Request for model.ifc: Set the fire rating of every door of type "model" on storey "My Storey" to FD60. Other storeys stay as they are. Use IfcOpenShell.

First a look at what the model holds.

```python
import ifcopenshell
import ifcopenshell.util.element

model = ifcopenshell.open("model.ifc")
print(model.schema)
storey = next(s for s in model.by_type("IfcBuildingStorey") if s.Name == "My Storey")
doors = [e for e in ifcopenshell.util.element.get_decomposition(storey) if e.is_a("IfcDoor")]
seen = {}
for e in doors:
    element_type = ifcopenshell.util.element.get_type(e)
    key = (element_type.Name if element_type != e and element_type else None, ifcopenshell.util.element.get_pset(e, "Pset_DoorCommon", "FireRating"))
    seen[key] = seen.get(key, 0) + 1
for (name, value), count in sorted(seen.items(), key=str):
    print(count, "x", name, "|", value)
```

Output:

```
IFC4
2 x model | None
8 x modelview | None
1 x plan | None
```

```python
import ifcopenshell
import ifcopenshell.api.pset
import ifcopenshell.util.element

model = ifcopenshell.open("model.ifc")

storey = next(s for s in model.by_type("IfcBuildingStorey") if s.Name == "My Storey")
doors = [e for e in ifcopenshell.util.element.get_decomposition(storey) if e.is_a("IfcDoor")]

count = 0
for e in doors:
    element_type = ifcopenshell.util.element.get_type(e)
    if element_type in (None, e) or element_type.Name != "model":
        continue
    # add_pset returns the element's existing set when there is one.
    pset = ifcopenshell.api.pset.add_pset(model, product=e, name="Pset_DoorCommon")
    ifcopenshell.api.pset.edit_pset(model, pset=pset, properties={"FireRating": "FD60"})
    count += 1

print(count, "doors updated")

model.write("model-out.ifc")
```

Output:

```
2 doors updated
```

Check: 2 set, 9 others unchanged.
